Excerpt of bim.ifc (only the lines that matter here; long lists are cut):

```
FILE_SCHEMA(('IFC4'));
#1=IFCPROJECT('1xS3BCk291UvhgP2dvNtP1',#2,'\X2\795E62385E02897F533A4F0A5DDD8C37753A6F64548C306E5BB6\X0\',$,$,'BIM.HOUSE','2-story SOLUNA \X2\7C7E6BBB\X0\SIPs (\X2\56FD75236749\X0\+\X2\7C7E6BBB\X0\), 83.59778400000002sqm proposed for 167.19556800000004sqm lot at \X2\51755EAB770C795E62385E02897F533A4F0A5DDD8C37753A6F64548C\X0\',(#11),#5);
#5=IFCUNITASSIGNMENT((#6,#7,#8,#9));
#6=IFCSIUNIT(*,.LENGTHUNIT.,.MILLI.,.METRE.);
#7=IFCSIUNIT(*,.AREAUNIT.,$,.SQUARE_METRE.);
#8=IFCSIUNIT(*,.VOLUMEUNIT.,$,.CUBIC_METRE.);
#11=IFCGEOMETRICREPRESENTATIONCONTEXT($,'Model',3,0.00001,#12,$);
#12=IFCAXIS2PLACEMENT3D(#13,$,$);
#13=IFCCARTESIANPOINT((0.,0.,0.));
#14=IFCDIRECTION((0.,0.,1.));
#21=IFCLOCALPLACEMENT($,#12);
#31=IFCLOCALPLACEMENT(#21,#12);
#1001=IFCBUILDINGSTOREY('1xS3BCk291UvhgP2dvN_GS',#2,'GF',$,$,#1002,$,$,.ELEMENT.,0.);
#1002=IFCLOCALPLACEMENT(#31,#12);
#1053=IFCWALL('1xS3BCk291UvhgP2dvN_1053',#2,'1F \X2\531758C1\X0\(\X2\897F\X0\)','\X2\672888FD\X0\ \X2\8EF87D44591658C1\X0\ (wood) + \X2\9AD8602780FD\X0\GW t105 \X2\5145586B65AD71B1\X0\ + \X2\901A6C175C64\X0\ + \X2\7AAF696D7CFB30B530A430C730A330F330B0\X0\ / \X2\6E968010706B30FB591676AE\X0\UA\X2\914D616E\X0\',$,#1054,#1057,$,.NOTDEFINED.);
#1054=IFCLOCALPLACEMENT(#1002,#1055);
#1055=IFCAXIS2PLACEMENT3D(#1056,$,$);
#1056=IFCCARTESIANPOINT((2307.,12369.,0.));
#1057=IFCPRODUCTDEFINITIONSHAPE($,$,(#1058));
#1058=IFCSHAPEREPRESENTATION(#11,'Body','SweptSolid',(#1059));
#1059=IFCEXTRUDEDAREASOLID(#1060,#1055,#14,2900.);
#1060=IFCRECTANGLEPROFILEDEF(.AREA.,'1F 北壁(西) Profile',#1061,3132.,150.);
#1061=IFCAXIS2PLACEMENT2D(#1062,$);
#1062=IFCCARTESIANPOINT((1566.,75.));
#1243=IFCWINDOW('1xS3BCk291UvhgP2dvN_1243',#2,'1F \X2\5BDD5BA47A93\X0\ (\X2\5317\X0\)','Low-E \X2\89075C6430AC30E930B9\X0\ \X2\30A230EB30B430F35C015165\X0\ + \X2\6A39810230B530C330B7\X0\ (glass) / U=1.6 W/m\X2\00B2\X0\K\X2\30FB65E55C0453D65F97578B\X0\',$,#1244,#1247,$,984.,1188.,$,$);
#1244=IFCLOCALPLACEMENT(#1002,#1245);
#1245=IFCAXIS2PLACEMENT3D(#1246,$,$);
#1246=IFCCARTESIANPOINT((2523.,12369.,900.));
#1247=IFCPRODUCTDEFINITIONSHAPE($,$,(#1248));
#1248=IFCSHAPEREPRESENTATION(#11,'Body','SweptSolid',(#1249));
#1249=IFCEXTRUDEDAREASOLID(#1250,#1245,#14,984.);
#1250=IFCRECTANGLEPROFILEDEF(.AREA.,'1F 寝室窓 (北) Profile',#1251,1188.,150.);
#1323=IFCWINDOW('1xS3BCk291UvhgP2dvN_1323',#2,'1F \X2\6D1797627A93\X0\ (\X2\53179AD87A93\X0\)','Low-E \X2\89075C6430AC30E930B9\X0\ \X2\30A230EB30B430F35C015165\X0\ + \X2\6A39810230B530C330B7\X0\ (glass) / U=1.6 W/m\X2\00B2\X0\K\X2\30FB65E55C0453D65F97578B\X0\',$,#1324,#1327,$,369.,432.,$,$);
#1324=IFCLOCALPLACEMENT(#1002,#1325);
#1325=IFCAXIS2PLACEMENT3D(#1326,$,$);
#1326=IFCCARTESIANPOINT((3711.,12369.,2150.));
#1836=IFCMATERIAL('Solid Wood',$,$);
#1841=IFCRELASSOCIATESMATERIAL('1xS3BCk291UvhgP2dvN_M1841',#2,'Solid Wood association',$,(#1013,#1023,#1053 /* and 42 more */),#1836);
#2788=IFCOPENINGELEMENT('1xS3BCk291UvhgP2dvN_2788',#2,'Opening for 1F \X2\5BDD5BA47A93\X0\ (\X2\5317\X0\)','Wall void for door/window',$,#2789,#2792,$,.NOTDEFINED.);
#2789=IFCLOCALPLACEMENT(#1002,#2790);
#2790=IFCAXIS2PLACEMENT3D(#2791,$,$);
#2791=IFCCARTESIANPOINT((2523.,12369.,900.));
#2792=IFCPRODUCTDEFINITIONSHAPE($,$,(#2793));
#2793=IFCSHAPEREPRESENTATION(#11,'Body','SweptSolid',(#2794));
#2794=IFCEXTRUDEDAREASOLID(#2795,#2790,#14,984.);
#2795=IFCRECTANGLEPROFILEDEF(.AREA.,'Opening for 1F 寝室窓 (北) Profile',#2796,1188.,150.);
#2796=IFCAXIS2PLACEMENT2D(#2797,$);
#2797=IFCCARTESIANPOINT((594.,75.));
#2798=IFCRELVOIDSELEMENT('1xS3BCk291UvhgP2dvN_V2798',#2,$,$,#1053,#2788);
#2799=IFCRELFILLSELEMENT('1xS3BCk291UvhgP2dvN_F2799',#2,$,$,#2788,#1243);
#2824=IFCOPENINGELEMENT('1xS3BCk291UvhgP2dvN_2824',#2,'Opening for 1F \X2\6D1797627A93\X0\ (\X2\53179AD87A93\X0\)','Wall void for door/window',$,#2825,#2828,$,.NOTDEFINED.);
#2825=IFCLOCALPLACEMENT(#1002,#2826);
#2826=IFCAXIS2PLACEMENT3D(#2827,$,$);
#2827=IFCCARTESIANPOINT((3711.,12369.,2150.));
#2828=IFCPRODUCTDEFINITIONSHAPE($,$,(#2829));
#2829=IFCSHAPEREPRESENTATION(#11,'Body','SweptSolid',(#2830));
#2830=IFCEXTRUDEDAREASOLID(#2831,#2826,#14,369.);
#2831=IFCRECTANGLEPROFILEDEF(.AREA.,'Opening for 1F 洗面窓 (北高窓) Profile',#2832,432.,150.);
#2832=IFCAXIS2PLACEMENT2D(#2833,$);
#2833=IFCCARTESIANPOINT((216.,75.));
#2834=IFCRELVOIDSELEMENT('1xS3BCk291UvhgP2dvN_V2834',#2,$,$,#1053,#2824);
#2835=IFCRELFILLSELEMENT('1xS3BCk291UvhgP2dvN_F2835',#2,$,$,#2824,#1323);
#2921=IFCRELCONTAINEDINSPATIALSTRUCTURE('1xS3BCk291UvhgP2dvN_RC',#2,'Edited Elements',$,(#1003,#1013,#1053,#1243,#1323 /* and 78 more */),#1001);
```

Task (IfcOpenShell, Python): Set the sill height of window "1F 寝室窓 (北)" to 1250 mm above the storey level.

```python
import numpy as np
import ifcopenshell
import ifcopenshell.api.geometry
import ifcopenshell.geom
import ifcopenshell.util.element
import ifcopenshell.util.placement
import ifcopenshell.util.shape
import ifcopenshell.util.unit

model = ifcopenshell.open("bim.ifc")
unit_scale = ifcopenshell.util.unit.calculate_unit_scale(model)

window = model.by_guid("1xS3BCk291UvhgP2dvN_1243")
opening = window.FillsVoids[0].RelatingOpeningElement
storey = ifcopenshell.util.element.get_container(window, ifc_class="IfcBuildingStorey")
level = ifcopenshell.util.placement.get_local_placement(storey.ObjectPlacement)[2, 3]

# The opening's origin need not be at the sill, so measure its lowest point.
shape = ifcopenshell.geom.create_shape(ifcopenshell.geom.settings(), opening)
bottom = ifcopenshell.util.shape.get_shape_bottom_elevation(shape, shape.geometry) / unit_scale
dz = level + 1.25 / unit_scale - bottom

shift = np.array([0.0, 0.0, dz])
# The window is not placed relative to its opening, so move both.
for product in (opening, window):
    matrix = ifcopenshell.util.placement.get_local_placement(product.ObjectPlacement)
    matrix[:3, 3] += shift
    ifcopenshell.api.geometry.edit_object_placement(model, product=product, matrix=matrix, is_si=False)

print(f"moved by {dz * unit_scale:+.3f} m")

model.write("bim_edited.ifc")
```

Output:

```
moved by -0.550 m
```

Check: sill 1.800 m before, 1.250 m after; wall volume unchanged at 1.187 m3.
